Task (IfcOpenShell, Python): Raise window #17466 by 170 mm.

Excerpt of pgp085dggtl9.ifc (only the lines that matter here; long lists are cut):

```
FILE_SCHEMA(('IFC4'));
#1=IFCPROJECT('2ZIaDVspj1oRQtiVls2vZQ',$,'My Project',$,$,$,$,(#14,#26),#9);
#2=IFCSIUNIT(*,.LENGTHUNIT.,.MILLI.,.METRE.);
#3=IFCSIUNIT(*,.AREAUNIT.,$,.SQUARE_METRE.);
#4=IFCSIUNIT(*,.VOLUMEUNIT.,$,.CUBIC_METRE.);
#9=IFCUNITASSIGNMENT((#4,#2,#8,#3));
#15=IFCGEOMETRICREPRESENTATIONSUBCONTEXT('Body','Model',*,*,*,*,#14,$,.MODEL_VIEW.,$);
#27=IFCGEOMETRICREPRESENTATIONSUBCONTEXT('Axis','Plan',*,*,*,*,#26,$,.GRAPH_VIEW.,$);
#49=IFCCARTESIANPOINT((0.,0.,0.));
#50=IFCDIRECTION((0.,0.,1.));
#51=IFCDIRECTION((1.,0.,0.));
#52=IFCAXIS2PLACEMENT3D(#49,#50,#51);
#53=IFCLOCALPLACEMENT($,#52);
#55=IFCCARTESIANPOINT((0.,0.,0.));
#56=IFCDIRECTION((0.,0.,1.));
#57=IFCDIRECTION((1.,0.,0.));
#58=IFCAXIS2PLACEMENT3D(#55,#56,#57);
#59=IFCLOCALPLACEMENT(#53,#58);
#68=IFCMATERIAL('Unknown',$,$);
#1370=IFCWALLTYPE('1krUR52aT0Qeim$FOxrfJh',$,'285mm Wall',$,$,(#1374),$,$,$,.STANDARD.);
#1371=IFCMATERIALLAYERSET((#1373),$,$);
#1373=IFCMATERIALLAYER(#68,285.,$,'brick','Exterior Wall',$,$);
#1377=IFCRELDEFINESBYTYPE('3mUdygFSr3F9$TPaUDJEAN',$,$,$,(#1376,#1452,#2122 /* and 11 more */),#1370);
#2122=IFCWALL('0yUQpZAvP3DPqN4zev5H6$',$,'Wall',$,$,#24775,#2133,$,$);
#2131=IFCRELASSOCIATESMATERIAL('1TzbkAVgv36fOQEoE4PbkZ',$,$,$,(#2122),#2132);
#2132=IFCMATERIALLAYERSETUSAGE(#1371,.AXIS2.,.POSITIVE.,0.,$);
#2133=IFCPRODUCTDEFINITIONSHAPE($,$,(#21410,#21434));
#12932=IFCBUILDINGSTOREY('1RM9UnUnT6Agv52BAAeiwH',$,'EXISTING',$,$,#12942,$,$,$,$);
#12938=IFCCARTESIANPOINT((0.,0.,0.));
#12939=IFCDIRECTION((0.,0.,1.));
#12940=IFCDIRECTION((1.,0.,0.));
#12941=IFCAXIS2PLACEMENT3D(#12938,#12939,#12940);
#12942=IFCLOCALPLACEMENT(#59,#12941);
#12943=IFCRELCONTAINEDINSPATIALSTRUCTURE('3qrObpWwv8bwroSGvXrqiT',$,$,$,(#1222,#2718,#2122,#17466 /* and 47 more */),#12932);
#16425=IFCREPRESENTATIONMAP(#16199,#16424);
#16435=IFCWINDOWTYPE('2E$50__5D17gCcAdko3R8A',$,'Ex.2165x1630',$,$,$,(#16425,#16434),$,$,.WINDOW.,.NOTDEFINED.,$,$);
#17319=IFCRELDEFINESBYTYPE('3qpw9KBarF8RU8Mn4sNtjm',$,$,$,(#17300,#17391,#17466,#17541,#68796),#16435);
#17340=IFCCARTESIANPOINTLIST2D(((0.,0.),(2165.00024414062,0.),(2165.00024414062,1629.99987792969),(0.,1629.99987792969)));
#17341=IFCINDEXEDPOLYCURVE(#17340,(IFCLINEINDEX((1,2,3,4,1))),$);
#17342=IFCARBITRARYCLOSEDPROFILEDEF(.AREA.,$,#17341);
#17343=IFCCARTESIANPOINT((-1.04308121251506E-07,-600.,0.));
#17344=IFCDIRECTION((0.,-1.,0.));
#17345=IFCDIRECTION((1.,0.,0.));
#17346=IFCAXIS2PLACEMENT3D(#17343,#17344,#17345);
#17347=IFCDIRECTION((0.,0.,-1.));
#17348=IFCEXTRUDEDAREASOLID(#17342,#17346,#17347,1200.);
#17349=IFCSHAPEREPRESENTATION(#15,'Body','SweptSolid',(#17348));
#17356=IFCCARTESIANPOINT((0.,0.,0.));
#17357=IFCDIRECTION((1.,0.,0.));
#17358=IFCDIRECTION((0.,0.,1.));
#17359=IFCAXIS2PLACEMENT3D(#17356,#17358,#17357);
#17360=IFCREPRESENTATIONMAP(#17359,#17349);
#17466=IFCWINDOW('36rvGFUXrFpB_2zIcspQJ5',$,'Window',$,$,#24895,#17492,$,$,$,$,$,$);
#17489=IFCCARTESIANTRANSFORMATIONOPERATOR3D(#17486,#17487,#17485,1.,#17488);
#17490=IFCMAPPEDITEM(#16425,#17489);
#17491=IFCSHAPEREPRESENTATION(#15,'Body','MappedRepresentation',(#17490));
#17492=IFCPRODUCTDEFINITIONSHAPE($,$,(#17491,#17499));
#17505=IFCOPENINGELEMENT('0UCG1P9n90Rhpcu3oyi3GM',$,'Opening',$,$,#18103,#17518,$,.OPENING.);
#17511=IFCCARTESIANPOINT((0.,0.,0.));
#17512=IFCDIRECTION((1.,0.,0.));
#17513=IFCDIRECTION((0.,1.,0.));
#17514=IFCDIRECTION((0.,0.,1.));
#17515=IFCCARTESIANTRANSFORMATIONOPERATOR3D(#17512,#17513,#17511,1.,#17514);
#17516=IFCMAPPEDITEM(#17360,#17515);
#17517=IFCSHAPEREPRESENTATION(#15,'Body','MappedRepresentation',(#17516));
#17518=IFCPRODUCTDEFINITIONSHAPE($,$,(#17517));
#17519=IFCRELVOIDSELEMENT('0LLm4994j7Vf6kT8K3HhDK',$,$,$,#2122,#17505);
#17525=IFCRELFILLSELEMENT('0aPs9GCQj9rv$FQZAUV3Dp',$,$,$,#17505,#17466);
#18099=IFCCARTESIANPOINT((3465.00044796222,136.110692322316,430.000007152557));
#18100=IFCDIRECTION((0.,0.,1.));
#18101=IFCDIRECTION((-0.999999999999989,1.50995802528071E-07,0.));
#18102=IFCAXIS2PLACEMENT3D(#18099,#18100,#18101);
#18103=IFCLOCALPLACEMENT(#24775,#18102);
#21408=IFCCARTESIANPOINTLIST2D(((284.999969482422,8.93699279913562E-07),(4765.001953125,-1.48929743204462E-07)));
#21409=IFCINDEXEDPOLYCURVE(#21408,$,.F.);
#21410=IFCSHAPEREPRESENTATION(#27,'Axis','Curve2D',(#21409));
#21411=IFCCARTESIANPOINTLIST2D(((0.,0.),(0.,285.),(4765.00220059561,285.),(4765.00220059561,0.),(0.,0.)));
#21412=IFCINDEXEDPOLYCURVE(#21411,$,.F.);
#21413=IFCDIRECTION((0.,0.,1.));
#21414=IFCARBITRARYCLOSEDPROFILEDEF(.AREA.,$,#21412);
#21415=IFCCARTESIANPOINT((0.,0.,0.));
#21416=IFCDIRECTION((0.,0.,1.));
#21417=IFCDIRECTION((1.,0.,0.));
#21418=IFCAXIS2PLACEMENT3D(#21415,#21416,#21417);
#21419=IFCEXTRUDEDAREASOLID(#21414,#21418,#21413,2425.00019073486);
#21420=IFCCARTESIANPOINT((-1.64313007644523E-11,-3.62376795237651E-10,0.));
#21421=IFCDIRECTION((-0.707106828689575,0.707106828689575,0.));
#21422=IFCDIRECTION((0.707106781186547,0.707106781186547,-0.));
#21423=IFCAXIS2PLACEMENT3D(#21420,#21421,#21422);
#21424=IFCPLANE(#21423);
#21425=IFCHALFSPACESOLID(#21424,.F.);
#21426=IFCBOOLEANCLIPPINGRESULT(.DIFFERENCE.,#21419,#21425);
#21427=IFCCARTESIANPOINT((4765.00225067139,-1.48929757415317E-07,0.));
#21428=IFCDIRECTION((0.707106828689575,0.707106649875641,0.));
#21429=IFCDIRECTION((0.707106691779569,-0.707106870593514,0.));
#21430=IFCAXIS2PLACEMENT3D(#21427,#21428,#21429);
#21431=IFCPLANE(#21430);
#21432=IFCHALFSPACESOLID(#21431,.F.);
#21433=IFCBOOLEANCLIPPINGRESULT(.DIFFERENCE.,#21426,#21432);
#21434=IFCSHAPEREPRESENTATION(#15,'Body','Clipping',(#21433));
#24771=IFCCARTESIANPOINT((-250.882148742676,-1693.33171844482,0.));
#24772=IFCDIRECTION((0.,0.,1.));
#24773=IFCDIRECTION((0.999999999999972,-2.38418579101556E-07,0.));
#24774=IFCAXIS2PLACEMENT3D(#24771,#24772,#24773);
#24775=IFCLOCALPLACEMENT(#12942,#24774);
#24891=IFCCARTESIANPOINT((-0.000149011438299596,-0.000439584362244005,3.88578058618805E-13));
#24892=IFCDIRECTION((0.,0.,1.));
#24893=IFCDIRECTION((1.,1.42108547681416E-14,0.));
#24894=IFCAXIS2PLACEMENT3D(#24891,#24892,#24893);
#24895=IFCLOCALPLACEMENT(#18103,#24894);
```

```python
import numpy as np
import ifcopenshell
import ifcopenshell.api.geometry
import ifcopenshell.util.placement
import ifcopenshell.util.unit

model = ifcopenshell.open("pgp085dggtl9.ifc")
unit_scale = ifcopenshell.util.unit.calculate_unit_scale(model)

window = model.by_guid("36rvGFUXrFpB_2zIcspQJ5")
opening = window.FillsVoids[0].RelatingOpeningElement
dz = 0.17 / unit_scale

shift = np.array([0.0, 0.0, dz])
# The window is placed relative to its opening, so it follows when the opening moves.
matrix = ifcopenshell.util.placement.get_local_placement(opening.ObjectPlacement)
matrix[:3, 3] += shift
ifcopenshell.api.geometry.edit_object_placement(
    model, product=opening, matrix=matrix, is_si=False, should_transform_children=True
)

print(f"moved by {dz * unit_scale:+.3f} m")

model.write("pgp085dggtl9_rev.ifc")
```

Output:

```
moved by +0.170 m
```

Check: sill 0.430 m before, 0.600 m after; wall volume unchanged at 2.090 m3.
